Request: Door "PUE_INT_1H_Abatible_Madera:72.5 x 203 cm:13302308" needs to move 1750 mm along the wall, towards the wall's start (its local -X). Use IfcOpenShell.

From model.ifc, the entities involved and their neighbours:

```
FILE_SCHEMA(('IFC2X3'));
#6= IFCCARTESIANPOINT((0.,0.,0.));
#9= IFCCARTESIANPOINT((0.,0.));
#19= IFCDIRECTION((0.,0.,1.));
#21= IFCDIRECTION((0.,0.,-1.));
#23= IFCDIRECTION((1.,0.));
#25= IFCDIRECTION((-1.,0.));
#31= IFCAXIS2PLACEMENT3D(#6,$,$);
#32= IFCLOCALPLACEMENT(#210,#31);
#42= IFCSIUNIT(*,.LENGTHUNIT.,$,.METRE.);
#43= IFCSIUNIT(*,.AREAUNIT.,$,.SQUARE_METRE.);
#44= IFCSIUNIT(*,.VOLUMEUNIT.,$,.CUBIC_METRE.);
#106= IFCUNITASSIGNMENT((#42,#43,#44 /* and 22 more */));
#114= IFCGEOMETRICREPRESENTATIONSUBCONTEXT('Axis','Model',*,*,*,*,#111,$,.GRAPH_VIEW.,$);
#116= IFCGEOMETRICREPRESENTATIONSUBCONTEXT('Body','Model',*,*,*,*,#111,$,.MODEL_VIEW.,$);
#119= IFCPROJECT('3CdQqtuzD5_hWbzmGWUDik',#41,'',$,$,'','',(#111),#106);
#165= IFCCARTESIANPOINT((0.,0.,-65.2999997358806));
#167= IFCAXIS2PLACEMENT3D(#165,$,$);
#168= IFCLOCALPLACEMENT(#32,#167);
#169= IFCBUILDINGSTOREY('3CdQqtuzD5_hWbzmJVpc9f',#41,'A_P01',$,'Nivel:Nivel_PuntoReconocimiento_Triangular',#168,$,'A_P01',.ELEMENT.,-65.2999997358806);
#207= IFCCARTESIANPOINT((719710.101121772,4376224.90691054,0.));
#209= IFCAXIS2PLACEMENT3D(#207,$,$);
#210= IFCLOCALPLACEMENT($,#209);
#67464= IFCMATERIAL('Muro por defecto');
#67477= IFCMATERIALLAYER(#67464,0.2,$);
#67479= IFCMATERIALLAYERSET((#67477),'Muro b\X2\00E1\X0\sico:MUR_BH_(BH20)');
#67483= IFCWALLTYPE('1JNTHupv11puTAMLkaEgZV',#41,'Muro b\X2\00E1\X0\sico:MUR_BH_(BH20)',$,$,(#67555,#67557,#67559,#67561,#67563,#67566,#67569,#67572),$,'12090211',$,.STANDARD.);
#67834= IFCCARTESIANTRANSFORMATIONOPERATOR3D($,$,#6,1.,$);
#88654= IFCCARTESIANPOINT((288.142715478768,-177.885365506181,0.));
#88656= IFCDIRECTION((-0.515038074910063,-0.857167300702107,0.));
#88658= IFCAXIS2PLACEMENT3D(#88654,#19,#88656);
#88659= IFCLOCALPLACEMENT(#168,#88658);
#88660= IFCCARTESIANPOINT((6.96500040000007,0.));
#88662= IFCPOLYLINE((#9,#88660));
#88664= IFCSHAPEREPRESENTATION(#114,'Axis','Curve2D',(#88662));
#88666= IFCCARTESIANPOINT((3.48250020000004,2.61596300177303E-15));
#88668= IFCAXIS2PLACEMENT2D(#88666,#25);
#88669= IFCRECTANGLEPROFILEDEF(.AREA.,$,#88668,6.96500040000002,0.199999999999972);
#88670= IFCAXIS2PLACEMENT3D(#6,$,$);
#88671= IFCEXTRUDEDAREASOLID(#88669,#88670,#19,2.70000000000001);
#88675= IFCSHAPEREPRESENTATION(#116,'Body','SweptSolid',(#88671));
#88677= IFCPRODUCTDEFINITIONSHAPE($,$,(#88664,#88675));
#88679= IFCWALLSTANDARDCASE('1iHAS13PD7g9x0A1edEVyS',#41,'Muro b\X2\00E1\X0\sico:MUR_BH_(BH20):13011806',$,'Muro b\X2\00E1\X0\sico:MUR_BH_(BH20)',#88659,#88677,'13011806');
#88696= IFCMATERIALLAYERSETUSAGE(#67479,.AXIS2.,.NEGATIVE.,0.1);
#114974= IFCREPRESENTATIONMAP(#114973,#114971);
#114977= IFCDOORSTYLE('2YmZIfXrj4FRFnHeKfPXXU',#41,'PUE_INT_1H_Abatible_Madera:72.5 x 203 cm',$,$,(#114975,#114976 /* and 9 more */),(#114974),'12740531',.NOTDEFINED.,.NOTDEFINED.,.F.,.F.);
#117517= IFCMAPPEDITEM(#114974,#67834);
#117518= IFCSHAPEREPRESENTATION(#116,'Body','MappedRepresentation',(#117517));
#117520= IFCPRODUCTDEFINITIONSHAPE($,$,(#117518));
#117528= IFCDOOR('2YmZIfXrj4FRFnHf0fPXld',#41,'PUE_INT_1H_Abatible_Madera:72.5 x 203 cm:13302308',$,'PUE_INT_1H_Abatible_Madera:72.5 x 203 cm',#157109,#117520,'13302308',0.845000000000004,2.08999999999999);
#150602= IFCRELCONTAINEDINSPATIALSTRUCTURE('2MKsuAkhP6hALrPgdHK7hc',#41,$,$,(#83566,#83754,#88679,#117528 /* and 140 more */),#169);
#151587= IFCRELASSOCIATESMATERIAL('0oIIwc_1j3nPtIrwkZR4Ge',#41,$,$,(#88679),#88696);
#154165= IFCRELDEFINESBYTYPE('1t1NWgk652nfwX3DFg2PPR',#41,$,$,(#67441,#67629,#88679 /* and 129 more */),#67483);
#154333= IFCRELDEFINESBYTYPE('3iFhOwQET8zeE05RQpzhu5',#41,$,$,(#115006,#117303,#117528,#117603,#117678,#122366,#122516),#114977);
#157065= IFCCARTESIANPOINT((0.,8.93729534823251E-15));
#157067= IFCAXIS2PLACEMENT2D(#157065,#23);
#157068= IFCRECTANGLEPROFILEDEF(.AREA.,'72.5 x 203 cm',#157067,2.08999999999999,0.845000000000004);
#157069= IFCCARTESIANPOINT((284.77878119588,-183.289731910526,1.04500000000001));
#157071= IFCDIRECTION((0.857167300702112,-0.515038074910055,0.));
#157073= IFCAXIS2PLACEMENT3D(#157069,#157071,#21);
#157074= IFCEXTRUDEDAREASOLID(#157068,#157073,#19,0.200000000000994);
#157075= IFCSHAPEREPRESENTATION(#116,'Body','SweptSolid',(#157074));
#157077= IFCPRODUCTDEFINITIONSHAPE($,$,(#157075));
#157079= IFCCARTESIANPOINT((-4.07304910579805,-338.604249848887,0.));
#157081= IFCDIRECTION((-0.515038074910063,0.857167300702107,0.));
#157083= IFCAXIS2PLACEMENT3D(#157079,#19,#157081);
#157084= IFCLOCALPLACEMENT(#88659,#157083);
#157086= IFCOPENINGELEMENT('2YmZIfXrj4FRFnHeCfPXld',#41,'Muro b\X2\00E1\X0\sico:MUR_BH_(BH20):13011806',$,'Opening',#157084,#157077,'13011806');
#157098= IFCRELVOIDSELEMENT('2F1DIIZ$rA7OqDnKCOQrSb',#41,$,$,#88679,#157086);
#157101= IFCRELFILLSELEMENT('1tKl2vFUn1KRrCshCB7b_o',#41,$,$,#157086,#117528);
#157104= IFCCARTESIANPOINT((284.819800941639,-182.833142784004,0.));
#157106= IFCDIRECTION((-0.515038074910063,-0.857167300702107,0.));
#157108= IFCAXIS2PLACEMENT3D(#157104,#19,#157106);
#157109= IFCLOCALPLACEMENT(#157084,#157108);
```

```python
import ifcopenshell
import ifcopenshell.api.geometry
import ifcopenshell.util.placement

model = ifcopenshell.open("model.ifc")

door = model.by_guid("2YmZIfXrj4FRFnHf0fPXld")
opening = door.FillsVoids[0].RelatingOpeningElement
wall = opening.VoidsElements[0].RelatingBuildingElement

wall_matrix = ifcopenshell.util.placement.get_local_placement(wall.ObjectPlacement)
shift = wall_matrix[:3, 0] * -1.75
before = ifcopenshell.util.placement.get_local_placement(door.ObjectPlacement)[:3, 3].copy()

# The door is placed relative to its opening, so it follows when the opening moves.
matrix = ifcopenshell.util.placement.get_local_placement(opening.ObjectPlacement)
matrix[:3, 3] += shift
ifcopenshell.api.geometry.edit_object_placement(
    model, product=opening, matrix=matrix, is_si=False, should_transform_children=True
)

after = ifcopenshell.util.placement.get_local_placement(door.ObjectPlacement)[:3, 3]
print("door moved by", (after - before).round(3) + 0.0)

model.write("model-out.ifc")
```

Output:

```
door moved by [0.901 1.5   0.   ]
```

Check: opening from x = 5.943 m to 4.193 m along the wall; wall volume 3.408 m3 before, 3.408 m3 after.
